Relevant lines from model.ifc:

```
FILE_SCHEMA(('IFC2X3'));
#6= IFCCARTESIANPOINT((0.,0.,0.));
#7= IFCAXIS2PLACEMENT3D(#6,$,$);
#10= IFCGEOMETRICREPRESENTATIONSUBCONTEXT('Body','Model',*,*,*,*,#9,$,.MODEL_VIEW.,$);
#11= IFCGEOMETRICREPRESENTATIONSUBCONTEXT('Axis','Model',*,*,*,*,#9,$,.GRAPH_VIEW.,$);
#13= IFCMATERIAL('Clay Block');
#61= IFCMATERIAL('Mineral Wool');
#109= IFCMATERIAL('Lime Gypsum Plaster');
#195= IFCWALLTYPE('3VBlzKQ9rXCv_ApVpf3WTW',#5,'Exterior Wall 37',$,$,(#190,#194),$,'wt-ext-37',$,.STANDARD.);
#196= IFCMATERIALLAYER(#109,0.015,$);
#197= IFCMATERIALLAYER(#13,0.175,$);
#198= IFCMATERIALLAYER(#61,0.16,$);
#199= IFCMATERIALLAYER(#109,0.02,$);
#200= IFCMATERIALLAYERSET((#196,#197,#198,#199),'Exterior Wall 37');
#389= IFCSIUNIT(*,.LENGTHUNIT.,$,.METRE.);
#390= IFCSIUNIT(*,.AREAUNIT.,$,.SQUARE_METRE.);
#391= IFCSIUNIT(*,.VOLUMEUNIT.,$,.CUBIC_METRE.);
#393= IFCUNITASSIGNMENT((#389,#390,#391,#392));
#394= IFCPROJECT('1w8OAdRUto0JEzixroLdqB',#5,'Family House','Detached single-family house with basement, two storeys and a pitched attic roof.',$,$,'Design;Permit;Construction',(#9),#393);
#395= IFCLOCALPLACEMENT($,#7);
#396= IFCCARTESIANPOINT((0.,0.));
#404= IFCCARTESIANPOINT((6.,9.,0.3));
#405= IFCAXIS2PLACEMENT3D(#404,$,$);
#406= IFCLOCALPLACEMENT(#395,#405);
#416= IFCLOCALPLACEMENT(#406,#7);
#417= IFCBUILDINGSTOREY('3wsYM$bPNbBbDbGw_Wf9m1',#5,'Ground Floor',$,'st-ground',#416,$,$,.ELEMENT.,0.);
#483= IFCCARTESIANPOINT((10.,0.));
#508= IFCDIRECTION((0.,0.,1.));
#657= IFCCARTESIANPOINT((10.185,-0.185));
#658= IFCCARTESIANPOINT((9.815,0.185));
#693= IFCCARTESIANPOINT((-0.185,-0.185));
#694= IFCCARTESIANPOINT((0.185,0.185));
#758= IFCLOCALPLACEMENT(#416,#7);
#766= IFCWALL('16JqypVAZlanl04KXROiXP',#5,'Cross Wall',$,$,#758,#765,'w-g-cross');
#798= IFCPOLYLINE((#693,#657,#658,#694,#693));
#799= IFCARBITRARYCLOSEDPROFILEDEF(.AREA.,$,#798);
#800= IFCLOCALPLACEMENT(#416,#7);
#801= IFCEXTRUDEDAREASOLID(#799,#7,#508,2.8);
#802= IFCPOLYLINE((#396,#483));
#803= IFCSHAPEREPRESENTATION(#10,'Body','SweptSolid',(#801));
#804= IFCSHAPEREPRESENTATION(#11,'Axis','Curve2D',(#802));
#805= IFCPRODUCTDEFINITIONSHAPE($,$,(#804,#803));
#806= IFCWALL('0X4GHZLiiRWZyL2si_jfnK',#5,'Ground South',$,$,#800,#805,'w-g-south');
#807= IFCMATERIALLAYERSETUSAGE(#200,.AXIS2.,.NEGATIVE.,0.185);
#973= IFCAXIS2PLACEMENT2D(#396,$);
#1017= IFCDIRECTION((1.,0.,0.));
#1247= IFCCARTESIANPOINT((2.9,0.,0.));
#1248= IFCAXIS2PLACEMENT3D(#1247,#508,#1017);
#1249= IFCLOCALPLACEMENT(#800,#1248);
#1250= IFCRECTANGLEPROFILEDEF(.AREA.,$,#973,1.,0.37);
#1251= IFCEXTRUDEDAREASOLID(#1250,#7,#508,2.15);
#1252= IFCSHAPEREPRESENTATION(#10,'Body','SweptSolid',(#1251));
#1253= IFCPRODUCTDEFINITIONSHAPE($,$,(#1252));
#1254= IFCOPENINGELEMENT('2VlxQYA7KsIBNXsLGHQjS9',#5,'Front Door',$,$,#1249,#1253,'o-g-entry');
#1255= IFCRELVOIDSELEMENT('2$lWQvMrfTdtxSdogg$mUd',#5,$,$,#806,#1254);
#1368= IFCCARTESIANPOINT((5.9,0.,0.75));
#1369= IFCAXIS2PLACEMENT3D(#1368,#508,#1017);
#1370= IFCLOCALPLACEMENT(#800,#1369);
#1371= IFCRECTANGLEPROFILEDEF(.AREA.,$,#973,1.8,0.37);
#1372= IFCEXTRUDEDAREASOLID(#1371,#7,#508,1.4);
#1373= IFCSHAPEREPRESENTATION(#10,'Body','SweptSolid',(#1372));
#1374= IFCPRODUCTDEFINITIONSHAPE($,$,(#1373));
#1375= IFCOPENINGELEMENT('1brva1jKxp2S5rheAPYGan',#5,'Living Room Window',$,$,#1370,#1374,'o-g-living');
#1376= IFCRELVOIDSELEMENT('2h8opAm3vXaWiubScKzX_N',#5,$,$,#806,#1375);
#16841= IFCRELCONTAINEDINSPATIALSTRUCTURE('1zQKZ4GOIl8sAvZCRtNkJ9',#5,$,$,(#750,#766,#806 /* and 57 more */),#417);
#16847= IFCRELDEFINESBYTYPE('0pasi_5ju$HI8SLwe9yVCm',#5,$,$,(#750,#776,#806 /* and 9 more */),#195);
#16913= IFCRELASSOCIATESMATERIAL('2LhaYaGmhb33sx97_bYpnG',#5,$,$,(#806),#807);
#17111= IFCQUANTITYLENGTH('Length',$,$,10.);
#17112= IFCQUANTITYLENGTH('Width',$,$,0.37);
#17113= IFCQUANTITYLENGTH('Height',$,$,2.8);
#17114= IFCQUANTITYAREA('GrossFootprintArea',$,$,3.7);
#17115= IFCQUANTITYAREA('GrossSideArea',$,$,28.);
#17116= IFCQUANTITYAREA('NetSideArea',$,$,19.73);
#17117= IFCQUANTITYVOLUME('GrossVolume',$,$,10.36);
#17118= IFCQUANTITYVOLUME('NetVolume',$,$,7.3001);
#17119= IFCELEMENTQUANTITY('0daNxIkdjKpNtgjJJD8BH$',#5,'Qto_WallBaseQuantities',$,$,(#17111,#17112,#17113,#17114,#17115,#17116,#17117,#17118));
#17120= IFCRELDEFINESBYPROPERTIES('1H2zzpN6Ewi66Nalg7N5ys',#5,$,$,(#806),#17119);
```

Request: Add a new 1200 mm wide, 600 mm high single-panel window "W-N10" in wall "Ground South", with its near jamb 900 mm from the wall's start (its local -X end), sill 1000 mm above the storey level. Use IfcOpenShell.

```python
import numpy as np
import ifcopenshell
import ifcopenshell.api.feature
import ifcopenshell.api.geometry
import ifcopenshell.api.pset
import ifcopenshell.api.root
import ifcopenshell.api.spatial
import ifcopenshell.api.type
import ifcopenshell.geom
import ifcopenshell.util.element
import ifcopenshell.util.placement
import ifcopenshell.util.representation
import ifcopenshell.util.shape
import ifcopenshell.util.unit

model = ifcopenshell.open("model.ifc")
unit_scale = ifcopenshell.util.unit.calculate_unit_scale(model)
area_scale = ifcopenshell.util.unit.calculate_unit_scale(model, "AREAUNIT")
volume_scale = ifcopenshell.util.unit.calculate_unit_scale(model, "VOLUMEUNIT")
settings = ifcopenshell.geom.settings()


def volume(element):
    """Net volume in cubic metres, openings subtracted."""
    shape = ifcopenshell.geom.create_shape(settings, element)
    return ifcopenshell.util.shape.get_volume(shape.geometry)


wall = model.by_guid("0X4GHZLiiRWZyL2si_jfnK")
storey = ifcopenshell.util.element.get_container(wall, ifc_class="IfcBuildingStorey")
context = ifcopenshell.util.representation.get_context(model, "Model", "Body", "MODEL_VIEW")
before = volume(wall)

width, height, from_end, sill = 1.2, 0.6, 0.9, 1  # metres

# The wall runs along its own X axis, and the end named is its -X end.
wall_shape = ifcopenshell.geom.create_shape(settings, wall)
x, y, z = ifcopenshell.util.shape.get_vertices(wall_shape.geometry).T
start = x.min() + from_end
face, thickness = float(y.min()), float(y.max() - y.min())
wall_matrix = ifcopenshell.util.placement.get_local_placement(wall.ObjectPlacement)
level = ifcopenshell.util.placement.get_local_placement(storey.ObjectPlacement)[2, 3]


def in_wall(x, y):
    """Placement at x, y metres in the wall's axes, at sill height."""
    matrix = wall_matrix.copy()
    matrix[:, 3] = wall_matrix @ np.array([x / unit_scale, y / unit_scale, 0.0, 1.0])
    matrix[2, 3] = level + sill / unit_scale
    return matrix


# Opening: a box that overshoots both wall faces by 50 mm.
opening = ifcopenshell.api.root.create_entity(model, ifc_class="IfcOpeningElement")
box = ifcopenshell.api.geometry.add_wall_representation(
    model, context=context, length=width, height=height, thickness=thickness + 0.1
)
ifcopenshell.api.geometry.assign_representation(model, product=opening, representation=box)
ifcopenshell.api.geometry.edit_object_placement(model, product=opening, matrix=in_wall(start, face - 0.05), is_si=False)
ifcopenshell.api.feature.add_feature(model, feature=opening, element=wall)

window = ifcopenshell.api.root.create_entity(model, ifc_class="IfcWindow", name="W-N10")
window.OverallWidth, window.OverallHeight = width / unit_scale, height / unit_scale
body = ifcopenshell.api.geometry.add_window_representation(
    model,
    context=context,
    overall_width=window.OverallWidth,
    overall_height=window.OverallHeight,
    partition_type="SINGLE_PANEL",
)
ifcopenshell.api.geometry.assign_representation(model, product=window, representation=body)
ifcopenshell.api.spatial.assign_container(model, products=[window], relating_structure=storey)
fills = ifcopenshell.api.feature.add_filling(model, opening=opening, element=window)
fills.OwnerHistory = window.OwnerHistory  # required in IFC2X3

# IFC2X3 keeps the operation on the window style.
style = ifcopenshell.api.root.create_entity(model, ifc_class="IfcWindowStyle", name="W-N10")
style.OperationType, style.ConstructionType = "SINGLE_PANEL", "NOTDEFINED"
style.ParameterTakesPrecedence = style.Sizeable = False
ifcopenshell.api.type.assign_type(model, related_objects=[window], relating_type=style)

# Centre the window in the wall's thickness.
ifcopenshell.api.geometry.edit_object_placement(model, product=window, matrix=in_wall(start, face), is_si=False)
window_shape = ifcopenshell.geom.create_shape(settings, window)
depth = ifcopenshell.util.shape.get_vertices(window_shape.geometry)[:, 1]
offset = face + thickness / 2 - (depth.min() + depth.max()) / 2
ifcopenshell.api.geometry.edit_object_placement(model, product=window, matrix=in_wall(start, offset), is_si=False)

after = volume(wall)

# Update the wall's stored quantities.
qto = model.by_id(ifcopenshell.util.element.get_pset(wall, "Qto_WallBaseQuantities", should_inherit=False)["id"])
ifcopenshell.api.pset.edit_qto(model, qto=qto, properties={
    "NetSideArea": after / thickness / area_scale,
    "NetVolume": after / volume_scale,
})

print(f"wall volume {before:.3f} -> {after:.3f} m3")

model.write("model_rev.ifc")
```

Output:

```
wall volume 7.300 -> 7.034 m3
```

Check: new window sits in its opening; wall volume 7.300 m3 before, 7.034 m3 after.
